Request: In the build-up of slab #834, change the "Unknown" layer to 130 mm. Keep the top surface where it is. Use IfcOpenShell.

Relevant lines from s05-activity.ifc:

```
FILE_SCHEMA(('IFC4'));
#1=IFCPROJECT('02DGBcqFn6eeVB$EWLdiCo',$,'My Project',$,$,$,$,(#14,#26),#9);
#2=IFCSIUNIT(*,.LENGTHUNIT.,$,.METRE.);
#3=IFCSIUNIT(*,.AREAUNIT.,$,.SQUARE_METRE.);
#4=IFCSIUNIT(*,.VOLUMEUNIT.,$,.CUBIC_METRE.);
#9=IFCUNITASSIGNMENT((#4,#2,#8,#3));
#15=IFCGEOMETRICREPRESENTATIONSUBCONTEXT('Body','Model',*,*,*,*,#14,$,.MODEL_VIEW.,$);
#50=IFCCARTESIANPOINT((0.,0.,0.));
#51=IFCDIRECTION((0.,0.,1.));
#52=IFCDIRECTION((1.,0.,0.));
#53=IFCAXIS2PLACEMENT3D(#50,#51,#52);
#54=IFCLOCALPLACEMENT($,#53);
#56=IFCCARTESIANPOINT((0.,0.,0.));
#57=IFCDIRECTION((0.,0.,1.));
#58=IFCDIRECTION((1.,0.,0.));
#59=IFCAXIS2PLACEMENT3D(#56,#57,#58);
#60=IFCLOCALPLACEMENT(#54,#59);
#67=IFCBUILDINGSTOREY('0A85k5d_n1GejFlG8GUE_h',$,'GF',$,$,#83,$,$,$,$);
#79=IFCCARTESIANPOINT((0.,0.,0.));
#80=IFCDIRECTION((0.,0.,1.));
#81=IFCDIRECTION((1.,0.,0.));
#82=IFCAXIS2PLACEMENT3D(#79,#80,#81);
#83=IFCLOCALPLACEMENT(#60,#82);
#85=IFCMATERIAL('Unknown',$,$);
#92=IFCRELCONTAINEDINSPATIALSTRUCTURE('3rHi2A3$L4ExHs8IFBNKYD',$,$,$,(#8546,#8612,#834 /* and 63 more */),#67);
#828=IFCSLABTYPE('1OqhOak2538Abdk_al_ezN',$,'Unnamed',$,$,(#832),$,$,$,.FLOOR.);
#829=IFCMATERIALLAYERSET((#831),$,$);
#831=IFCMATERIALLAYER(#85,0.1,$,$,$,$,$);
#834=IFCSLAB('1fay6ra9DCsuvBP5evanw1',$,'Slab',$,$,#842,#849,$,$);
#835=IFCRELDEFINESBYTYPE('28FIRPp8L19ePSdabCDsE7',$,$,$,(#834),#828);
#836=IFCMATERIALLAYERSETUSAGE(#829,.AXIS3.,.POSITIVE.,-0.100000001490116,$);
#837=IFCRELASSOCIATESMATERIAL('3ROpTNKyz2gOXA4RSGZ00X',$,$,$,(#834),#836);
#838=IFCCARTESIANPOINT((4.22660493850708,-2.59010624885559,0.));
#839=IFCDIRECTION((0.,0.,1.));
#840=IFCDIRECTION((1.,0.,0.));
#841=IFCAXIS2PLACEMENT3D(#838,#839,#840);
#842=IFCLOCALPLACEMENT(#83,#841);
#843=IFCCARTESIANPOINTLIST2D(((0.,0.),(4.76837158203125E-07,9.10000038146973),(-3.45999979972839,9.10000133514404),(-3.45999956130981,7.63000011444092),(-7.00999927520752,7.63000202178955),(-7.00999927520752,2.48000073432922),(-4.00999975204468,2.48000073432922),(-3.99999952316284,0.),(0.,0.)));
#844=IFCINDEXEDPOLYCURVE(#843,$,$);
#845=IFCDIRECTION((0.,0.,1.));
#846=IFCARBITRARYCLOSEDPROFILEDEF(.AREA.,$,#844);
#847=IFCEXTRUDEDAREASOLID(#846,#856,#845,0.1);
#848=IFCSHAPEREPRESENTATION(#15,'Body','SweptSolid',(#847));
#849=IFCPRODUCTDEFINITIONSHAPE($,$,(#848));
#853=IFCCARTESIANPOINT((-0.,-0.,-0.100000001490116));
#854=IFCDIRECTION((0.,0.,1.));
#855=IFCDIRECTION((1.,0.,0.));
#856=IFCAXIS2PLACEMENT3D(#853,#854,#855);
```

```python
import ifcopenshell
import ifcopenshell.util.element
import ifcopenshell.util.representation
import ifcopenshell.util.unit

model = ifcopenshell.open("s05-activity.ifc")
unit_scale = ifcopenshell.util.unit.calculate_unit_scale(model)

layer_set = model.by_id(829)
layer = next(l for l in layer_set.MaterialLayers if l.Material and l.Material.Name == "Unknown")
change = 0.13 / unit_scale - layer.LayerThickness
layer.LayerThickness += change

# Geometry does not follow the layer set by itself.
slabs = [e for e in ifcopenshell.util.element.get_elements_by_material(model, layer_set) if e.is_a("IfcSlab")]
for slab in sorted(slabs, key=lambda e: e.id()):
    body = ifcopenshell.util.representation.get_representation(slab, "Model", "Body")
    solid = body.Items[0]
    old_depth = solid.Depth
    solid.Depth += change
    # Extruded upwards: lower the start of the extrusion so the top stays.
    x, y, z = solid.Position.Location.Coordinates
    solid.Position.Location = model.createIfcCartesianPoint((x, y, z - change))
    print(slab.id(), f"{old_depth:g} -> {solid.Depth:g}")

# The layers are counted up from the underside, which has moved.
for usage in {ifcopenshell.util.element.get_material(slab) for slab in slabs}:
    usage.OffsetFromReferenceLine -= change

model.write("s05-activity-out.ifc")
```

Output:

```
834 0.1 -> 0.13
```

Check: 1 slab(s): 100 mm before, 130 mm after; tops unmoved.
